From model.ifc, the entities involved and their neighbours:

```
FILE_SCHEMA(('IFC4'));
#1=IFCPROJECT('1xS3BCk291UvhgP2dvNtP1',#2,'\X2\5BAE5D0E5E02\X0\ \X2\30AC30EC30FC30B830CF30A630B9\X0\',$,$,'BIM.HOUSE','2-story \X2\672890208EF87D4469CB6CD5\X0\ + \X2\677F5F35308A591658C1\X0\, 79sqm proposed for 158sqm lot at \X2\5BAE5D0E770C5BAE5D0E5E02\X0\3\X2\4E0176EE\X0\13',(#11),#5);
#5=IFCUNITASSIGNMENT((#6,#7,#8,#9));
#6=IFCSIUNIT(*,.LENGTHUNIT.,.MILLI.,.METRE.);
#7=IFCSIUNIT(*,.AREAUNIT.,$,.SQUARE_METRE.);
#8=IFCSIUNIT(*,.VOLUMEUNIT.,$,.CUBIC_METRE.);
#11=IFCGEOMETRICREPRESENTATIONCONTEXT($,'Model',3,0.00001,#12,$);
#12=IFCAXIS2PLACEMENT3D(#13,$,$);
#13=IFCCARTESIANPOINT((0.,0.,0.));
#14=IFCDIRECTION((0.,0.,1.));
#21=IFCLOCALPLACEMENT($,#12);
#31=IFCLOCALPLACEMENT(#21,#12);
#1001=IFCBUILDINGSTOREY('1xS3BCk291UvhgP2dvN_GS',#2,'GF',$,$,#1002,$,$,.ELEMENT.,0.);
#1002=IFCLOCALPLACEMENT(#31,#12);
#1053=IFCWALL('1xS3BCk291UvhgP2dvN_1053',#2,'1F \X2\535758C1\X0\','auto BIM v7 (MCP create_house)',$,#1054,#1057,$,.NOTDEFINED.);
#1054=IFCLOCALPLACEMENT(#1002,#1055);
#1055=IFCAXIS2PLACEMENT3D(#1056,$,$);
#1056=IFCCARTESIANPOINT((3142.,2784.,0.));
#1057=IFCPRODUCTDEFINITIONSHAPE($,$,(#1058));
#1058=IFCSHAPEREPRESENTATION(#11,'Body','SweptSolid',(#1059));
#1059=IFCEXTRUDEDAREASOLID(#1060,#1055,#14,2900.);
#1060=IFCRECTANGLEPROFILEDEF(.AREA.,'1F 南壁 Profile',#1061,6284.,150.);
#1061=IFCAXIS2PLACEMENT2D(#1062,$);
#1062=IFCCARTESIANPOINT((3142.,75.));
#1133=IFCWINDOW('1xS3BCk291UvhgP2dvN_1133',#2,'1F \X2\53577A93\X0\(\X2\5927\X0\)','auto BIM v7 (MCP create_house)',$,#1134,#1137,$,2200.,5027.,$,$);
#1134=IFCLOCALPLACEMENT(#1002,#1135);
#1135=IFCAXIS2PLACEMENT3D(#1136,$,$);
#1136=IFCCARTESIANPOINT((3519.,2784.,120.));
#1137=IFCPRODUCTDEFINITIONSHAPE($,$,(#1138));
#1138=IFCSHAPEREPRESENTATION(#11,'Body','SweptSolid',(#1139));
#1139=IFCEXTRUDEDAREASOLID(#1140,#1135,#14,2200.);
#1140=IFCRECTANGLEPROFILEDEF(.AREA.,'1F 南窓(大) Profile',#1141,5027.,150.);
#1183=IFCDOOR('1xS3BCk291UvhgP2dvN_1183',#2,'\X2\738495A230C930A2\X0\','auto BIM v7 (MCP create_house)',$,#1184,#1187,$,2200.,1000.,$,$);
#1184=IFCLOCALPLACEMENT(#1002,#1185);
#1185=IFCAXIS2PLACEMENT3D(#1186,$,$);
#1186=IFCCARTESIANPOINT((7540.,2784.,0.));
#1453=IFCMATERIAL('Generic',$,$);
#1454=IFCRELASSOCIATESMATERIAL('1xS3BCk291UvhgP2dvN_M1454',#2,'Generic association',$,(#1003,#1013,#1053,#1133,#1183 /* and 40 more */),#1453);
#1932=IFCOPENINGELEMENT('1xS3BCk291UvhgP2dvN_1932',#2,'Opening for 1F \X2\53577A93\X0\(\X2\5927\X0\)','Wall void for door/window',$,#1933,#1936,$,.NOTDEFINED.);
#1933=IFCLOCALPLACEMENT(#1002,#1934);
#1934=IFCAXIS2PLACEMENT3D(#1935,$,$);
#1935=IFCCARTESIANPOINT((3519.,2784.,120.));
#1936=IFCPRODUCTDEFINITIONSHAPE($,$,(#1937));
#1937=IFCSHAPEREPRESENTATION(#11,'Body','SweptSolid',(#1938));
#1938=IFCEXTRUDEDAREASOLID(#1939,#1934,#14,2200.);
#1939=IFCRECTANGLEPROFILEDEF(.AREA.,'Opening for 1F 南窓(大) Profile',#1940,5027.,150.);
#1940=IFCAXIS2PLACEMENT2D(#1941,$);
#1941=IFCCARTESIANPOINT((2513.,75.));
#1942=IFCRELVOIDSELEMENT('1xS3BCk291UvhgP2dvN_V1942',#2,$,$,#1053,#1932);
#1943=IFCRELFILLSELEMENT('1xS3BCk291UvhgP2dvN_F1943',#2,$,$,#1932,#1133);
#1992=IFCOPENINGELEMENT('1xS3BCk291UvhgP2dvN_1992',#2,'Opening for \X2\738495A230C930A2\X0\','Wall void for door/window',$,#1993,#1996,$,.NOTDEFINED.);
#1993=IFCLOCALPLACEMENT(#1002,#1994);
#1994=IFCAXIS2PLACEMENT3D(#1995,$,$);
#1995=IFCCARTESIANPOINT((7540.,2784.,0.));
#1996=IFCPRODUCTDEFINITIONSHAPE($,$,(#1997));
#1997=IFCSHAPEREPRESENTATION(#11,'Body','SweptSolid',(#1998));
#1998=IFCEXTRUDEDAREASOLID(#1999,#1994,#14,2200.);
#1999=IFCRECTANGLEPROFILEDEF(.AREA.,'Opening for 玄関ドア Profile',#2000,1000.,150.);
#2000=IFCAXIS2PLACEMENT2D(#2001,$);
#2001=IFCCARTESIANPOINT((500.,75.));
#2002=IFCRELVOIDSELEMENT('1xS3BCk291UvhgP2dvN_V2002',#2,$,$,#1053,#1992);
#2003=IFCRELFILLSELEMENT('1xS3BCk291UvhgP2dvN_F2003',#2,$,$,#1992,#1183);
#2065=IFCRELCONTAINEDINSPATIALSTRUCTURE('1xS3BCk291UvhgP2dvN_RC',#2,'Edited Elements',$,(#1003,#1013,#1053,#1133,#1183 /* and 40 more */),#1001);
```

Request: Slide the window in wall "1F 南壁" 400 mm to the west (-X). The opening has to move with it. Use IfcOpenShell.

```python
import ifcopenshell
import ifcopenshell.api.geometry
import ifcopenshell.util.placement
import ifcopenshell.util.unit

model = ifcopenshell.open("model.ifc")
unit_scale = ifcopenshell.util.unit.calculate_unit_scale(model)

window = model.by_guid("1xS3BCk291UvhgP2dvN_1133")
opening = window.FillsVoids[0].RelatingOpeningElement
wall = opening.VoidsElements[0].RelatingBuildingElement

wall_matrix = ifcopenshell.util.placement.get_local_placement(wall.ObjectPlacement)
shift = wall_matrix[:3, 0] * -0.4 / unit_scale
before = ifcopenshell.util.placement.get_local_placement(window.ObjectPlacement)[:3, 3].copy()

# The window is not placed relative to its opening, so move both.
for product in (opening, window):
    matrix = ifcopenshell.util.placement.get_local_placement(product.ObjectPlacement)
    matrix[:3, 3] += shift
    ifcopenshell.api.geometry.edit_object_placement(model, product=product, matrix=matrix, is_si=False)

after = ifcopenshell.util.placement.get_local_placement(window.ObjectPlacement)[:3, 3]
print("window moved by", (after - before).round(3) + 0.0)

model.write("model_edited.ifc")
```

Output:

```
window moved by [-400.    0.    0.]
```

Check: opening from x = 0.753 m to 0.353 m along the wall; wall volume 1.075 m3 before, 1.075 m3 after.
